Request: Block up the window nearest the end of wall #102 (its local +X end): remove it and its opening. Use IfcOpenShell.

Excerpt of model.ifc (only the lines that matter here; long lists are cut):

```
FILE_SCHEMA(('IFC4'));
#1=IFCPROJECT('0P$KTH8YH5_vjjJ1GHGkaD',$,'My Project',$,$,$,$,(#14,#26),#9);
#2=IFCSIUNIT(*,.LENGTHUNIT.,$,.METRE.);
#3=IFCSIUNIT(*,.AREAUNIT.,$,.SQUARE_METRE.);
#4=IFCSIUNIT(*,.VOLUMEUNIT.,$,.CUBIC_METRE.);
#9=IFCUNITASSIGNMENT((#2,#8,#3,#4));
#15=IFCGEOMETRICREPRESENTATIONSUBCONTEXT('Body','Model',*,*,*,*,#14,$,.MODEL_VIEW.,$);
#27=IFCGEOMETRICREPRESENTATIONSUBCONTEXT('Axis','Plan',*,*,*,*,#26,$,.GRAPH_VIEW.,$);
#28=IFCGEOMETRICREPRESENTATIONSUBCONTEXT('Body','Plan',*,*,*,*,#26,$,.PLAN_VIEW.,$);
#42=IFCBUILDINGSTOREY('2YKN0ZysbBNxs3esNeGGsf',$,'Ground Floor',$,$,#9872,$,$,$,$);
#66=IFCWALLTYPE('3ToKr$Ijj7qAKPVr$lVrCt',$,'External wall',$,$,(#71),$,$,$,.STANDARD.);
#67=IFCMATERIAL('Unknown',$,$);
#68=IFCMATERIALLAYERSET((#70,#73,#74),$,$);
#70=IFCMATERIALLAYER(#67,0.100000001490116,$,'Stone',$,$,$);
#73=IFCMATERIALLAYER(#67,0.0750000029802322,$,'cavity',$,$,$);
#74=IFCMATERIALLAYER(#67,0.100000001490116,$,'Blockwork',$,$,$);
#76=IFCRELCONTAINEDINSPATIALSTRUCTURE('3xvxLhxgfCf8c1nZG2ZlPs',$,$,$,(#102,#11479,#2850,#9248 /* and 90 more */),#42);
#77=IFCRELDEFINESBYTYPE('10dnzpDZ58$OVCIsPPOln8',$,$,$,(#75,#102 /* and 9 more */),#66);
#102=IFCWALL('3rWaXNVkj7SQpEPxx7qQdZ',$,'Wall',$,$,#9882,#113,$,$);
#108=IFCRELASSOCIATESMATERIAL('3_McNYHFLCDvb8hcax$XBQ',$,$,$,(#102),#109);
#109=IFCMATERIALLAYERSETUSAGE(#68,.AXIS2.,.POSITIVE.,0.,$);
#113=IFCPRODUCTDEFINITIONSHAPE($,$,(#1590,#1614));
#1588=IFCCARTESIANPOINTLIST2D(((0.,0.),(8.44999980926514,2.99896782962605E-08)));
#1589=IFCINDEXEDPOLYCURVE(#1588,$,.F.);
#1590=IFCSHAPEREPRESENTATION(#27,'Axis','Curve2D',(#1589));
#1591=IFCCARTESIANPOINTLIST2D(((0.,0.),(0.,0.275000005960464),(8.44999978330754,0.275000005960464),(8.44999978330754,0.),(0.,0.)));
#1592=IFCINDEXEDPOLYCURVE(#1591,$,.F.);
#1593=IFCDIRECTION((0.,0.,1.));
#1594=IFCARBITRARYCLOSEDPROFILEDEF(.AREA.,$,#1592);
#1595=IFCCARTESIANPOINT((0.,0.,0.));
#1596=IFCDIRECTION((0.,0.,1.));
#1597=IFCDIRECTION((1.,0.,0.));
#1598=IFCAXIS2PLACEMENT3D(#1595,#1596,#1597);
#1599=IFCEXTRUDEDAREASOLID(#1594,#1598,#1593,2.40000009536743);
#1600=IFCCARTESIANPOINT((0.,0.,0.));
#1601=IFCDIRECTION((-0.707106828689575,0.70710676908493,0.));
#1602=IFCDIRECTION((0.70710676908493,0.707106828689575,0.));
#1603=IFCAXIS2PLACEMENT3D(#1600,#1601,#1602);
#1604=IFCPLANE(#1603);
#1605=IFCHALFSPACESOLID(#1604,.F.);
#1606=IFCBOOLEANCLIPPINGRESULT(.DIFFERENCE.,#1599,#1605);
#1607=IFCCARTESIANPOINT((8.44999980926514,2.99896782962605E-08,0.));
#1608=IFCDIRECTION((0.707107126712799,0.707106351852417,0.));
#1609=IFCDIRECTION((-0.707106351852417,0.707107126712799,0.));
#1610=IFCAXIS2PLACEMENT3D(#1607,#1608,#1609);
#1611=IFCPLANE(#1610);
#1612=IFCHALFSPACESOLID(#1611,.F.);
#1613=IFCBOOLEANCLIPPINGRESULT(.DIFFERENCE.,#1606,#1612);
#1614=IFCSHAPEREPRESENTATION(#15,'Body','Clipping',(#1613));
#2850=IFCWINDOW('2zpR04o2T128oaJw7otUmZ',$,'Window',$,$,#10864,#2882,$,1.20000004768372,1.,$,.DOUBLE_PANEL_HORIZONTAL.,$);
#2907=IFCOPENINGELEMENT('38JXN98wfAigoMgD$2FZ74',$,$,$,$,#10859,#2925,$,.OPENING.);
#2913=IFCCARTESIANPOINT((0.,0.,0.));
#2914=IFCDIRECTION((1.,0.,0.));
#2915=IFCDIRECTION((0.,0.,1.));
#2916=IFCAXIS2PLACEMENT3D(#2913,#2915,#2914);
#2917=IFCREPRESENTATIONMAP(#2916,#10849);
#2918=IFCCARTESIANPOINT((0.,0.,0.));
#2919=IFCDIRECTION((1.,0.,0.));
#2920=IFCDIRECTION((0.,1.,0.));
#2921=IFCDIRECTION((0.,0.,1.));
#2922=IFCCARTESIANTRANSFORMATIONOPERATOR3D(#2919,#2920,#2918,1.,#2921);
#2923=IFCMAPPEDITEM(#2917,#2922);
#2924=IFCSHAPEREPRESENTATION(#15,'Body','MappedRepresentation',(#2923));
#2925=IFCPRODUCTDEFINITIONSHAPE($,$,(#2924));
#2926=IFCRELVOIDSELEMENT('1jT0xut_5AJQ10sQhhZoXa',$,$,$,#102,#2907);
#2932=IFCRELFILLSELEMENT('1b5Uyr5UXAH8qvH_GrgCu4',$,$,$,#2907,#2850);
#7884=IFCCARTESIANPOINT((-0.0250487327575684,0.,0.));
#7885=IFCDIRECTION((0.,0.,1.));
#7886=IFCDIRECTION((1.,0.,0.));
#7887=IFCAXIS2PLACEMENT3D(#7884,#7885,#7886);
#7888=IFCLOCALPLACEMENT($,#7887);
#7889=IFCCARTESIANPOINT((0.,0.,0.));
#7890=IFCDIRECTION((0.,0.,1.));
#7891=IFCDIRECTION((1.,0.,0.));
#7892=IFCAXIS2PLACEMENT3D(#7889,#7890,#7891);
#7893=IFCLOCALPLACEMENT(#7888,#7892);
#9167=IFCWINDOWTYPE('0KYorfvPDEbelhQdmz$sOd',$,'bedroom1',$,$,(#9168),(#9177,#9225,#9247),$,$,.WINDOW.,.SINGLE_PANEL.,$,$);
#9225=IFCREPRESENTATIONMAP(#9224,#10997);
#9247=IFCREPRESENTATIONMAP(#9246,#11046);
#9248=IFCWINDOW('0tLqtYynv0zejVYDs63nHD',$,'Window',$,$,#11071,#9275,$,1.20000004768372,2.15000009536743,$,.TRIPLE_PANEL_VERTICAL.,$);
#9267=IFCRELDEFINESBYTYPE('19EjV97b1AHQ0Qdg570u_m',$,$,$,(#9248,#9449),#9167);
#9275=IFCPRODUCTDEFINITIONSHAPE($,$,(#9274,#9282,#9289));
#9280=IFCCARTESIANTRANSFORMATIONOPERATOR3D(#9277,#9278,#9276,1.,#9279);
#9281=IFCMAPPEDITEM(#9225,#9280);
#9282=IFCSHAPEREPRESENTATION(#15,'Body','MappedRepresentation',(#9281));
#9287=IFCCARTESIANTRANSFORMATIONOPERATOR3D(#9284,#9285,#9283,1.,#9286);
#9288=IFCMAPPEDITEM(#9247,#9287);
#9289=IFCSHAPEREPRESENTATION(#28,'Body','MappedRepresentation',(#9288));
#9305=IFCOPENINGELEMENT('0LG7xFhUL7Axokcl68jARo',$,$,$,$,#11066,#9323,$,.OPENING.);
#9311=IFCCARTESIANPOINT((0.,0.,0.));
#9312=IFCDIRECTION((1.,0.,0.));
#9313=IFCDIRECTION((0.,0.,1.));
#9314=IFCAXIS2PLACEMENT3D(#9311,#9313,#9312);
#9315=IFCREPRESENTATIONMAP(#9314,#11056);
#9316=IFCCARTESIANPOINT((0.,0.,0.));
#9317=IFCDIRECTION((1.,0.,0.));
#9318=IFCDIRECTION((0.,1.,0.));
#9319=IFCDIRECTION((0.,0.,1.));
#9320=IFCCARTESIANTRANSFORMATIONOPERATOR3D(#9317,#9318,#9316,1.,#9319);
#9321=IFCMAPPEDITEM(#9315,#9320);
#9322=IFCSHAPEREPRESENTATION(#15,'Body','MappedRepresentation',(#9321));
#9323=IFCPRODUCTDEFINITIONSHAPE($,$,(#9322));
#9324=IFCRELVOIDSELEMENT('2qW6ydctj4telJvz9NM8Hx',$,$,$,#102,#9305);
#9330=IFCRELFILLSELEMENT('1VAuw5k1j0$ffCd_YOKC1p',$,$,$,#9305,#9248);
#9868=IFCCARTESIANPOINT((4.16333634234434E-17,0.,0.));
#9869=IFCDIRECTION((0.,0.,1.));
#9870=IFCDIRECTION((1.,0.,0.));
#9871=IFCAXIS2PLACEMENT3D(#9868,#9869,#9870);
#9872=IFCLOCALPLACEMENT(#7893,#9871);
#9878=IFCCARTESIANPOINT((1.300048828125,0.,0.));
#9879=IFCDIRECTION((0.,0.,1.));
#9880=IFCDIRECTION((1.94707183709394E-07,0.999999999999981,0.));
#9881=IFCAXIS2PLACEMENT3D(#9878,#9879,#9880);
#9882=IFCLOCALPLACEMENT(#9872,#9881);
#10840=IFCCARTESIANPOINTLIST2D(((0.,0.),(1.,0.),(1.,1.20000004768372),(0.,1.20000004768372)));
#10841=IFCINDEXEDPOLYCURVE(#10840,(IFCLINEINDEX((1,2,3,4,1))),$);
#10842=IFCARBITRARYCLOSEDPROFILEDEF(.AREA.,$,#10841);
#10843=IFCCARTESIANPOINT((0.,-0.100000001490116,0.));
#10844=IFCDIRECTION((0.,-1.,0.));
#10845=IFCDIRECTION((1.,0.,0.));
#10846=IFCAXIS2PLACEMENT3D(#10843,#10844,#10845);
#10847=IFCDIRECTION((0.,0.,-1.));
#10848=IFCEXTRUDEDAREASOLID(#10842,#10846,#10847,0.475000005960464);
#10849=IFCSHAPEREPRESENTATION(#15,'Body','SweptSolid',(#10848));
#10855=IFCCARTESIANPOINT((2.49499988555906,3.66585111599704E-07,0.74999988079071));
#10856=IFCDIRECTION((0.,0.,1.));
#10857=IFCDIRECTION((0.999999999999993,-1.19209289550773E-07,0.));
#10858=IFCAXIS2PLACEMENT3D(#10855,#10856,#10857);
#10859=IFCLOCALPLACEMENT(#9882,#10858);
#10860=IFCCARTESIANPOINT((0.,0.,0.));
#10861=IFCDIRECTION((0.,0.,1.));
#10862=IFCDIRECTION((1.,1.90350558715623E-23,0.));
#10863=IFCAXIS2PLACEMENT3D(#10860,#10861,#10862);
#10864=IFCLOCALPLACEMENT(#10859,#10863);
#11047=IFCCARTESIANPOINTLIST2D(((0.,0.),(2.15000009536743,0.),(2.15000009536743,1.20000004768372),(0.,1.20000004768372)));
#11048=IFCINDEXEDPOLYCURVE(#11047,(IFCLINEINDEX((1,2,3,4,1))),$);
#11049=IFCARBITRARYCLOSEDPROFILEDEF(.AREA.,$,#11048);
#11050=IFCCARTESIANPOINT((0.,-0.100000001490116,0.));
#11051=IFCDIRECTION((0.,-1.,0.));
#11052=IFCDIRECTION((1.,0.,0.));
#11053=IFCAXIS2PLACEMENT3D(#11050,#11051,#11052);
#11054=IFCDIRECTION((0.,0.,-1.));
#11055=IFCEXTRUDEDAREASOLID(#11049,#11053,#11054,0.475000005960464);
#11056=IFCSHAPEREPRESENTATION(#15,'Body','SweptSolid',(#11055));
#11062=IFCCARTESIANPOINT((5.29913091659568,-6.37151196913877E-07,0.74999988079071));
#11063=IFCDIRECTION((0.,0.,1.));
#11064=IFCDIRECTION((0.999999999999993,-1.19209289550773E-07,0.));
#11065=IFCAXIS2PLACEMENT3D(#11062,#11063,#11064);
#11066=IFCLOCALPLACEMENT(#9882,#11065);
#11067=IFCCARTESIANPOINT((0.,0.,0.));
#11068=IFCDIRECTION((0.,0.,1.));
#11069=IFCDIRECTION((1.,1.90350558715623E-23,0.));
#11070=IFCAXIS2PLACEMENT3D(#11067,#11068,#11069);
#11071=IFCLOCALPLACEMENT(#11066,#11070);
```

```python
import ifcopenshell
import ifcopenshell.api.feature
import ifcopenshell.api.root
import ifcopenshell.geom
import ifcopenshell.util.shape

model = ifcopenshell.open("model.ifc")
settings = ifcopenshell.geom.settings()


def volume(element):
    """Net volume in cubic metres, openings subtracted."""
    shape = ifcopenshell.geom.create_shape(settings, element)
    return ifcopenshell.util.shape.get_volume(shape.geometry)


window = model.by_guid("0tLqtYynv0zejVYDs63nHD")
opening = window.FillsVoids[0].RelatingOpeningElement
wall = opening.VoidsElements[0].RelatingBuildingElement
before = volume(wall)

ifcopenshell.api.root.remove_product(model, product=window)
ifcopenshell.api.feature.remove_feature(model, feature=opening)

after = volume(wall)

print(f"wall volume {before:.3f} -> {after:.3f} m3")

model.write("model_edited.ifc")
```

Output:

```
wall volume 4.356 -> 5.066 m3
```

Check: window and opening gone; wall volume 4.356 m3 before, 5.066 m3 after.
